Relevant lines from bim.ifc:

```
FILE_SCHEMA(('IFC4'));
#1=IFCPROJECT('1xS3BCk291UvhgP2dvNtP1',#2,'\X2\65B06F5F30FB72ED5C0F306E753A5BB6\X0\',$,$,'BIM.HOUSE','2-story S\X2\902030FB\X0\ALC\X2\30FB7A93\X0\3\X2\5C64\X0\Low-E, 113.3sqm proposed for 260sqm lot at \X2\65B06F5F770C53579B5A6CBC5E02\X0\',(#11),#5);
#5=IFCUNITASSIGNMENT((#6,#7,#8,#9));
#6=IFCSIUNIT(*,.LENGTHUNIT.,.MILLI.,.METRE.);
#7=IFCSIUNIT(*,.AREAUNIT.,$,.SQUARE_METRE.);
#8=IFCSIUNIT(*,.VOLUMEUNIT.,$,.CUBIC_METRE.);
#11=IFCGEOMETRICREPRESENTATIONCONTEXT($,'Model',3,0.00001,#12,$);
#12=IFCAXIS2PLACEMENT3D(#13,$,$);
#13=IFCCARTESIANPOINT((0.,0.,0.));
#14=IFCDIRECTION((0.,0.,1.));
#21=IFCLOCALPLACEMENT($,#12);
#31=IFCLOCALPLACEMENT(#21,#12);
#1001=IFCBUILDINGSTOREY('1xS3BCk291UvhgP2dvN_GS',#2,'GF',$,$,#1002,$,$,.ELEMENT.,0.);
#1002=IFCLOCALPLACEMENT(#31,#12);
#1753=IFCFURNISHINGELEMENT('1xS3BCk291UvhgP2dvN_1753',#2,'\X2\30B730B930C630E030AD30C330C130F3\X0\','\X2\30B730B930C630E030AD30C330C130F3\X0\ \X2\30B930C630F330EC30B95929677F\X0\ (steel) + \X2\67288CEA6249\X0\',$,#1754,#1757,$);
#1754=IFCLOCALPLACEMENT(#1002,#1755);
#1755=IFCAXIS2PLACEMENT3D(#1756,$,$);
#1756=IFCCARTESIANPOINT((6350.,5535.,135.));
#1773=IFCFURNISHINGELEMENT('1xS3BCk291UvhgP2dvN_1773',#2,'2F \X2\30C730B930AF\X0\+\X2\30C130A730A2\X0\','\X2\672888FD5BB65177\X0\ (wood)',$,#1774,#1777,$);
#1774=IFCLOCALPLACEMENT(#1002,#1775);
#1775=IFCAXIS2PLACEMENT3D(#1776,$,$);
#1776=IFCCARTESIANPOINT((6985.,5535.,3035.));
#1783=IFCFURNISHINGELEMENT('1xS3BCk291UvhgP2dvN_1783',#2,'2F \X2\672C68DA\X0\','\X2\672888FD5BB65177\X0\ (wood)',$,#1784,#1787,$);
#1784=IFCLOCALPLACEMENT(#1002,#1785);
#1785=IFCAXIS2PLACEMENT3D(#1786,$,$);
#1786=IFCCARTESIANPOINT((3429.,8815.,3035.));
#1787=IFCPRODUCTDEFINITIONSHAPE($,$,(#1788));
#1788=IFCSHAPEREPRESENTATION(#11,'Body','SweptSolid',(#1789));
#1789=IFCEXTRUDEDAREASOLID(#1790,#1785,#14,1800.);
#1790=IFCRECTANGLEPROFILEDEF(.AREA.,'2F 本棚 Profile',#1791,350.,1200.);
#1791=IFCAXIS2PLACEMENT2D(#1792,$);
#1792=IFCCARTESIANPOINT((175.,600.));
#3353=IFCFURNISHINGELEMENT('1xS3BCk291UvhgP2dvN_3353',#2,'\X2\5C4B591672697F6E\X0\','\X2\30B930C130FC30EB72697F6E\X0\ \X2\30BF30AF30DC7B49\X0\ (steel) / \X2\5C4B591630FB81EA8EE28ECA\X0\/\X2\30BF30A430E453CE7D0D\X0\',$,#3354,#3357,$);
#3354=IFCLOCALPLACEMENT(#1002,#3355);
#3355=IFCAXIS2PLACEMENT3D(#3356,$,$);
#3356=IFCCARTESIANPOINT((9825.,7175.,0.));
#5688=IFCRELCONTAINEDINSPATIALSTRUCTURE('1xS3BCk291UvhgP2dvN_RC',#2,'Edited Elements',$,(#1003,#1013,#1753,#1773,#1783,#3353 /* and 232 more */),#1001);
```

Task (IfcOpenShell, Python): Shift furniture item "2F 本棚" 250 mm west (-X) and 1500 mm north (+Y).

```python
import ifcopenshell
import ifcopenshell.api.geometry
import ifcopenshell.util.placement
import ifcopenshell.util.unit

model = ifcopenshell.open("bim.ifc")
unit_scale = ifcopenshell.util.unit.calculate_unit_scale(model)

item = model.by_guid("1xS3BCk291UvhgP2dvN_1783")
matrix = ifcopenshell.util.placement.get_local_placement(item.ObjectPlacement)
matrix[0, 3] -= 0.25 / unit_scale
matrix[1, 3] += 1.5 / unit_scale
ifcopenshell.api.geometry.edit_object_placement(model, product=item, matrix=matrix, is_si=False)

print(ifcopenshell.util.placement.get_local_placement(item.ObjectPlacement).round(3) + 0.0)

model.write("bim_rev.ifc")
```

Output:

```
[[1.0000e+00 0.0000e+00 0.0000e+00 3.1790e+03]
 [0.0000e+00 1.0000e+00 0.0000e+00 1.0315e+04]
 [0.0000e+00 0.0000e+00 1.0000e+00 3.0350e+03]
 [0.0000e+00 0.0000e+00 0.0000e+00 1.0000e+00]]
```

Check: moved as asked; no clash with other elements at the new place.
